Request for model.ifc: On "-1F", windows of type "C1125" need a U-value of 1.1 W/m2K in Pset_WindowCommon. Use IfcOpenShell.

First a look at what the model holds.

```python
import ifcopenshell
import ifcopenshell.util.element

model = ifcopenshell.open("model.ifc")
print(model.schema)
storey = next(s for s in model.by_type("IfcBuildingStorey") if s.Name == "-1F")
windows = [e for e in ifcopenshell.util.element.get_decomposition(storey) if e.is_a("IfcWindow")]
seen = {}
for e in windows:
    element_type = ifcopenshell.util.element.get_type(e)
    key = (element_type.Name if element_type != e and element_type else None, ifcopenshell.util.element.get_pset(e, "Pset_WindowCommon", "ThermalTransmittance"))
    seen[key] = seen.get(key, 0) + 1
for (name, value), count in sorted(seen.items(), key=str):
    print(count, "x", name, "|", value)
```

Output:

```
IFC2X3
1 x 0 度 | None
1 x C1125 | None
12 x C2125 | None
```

```python
import ifcopenshell
import ifcopenshell.api.pset
import ifcopenshell.util.element

model = ifcopenshell.open("model.ifc")

storey = next(s for s in model.by_type("IfcBuildingStorey") if s.Name == "-1F")
windows = [e for e in ifcopenshell.util.element.get_decomposition(storey) if e.is_a("IfcWindow")]

count = 0
for e in windows:
    element_type = ifcopenshell.util.element.get_type(e)
    if element_type in (None, e) or element_type.Name != "C1125":
        continue
    # add_pset returns the element's existing set when there is one.
    pset = ifcopenshell.api.pset.add_pset(model, product=e, name="Pset_WindowCommon")
    ifcopenshell.api.pset.edit_pset(model, pset=pset, properties={"ThermalTransmittance": 1.1})
    count += 1

print(count, "windows updated")

model.write("model_v2.ifc")
```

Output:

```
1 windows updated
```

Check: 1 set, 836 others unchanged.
